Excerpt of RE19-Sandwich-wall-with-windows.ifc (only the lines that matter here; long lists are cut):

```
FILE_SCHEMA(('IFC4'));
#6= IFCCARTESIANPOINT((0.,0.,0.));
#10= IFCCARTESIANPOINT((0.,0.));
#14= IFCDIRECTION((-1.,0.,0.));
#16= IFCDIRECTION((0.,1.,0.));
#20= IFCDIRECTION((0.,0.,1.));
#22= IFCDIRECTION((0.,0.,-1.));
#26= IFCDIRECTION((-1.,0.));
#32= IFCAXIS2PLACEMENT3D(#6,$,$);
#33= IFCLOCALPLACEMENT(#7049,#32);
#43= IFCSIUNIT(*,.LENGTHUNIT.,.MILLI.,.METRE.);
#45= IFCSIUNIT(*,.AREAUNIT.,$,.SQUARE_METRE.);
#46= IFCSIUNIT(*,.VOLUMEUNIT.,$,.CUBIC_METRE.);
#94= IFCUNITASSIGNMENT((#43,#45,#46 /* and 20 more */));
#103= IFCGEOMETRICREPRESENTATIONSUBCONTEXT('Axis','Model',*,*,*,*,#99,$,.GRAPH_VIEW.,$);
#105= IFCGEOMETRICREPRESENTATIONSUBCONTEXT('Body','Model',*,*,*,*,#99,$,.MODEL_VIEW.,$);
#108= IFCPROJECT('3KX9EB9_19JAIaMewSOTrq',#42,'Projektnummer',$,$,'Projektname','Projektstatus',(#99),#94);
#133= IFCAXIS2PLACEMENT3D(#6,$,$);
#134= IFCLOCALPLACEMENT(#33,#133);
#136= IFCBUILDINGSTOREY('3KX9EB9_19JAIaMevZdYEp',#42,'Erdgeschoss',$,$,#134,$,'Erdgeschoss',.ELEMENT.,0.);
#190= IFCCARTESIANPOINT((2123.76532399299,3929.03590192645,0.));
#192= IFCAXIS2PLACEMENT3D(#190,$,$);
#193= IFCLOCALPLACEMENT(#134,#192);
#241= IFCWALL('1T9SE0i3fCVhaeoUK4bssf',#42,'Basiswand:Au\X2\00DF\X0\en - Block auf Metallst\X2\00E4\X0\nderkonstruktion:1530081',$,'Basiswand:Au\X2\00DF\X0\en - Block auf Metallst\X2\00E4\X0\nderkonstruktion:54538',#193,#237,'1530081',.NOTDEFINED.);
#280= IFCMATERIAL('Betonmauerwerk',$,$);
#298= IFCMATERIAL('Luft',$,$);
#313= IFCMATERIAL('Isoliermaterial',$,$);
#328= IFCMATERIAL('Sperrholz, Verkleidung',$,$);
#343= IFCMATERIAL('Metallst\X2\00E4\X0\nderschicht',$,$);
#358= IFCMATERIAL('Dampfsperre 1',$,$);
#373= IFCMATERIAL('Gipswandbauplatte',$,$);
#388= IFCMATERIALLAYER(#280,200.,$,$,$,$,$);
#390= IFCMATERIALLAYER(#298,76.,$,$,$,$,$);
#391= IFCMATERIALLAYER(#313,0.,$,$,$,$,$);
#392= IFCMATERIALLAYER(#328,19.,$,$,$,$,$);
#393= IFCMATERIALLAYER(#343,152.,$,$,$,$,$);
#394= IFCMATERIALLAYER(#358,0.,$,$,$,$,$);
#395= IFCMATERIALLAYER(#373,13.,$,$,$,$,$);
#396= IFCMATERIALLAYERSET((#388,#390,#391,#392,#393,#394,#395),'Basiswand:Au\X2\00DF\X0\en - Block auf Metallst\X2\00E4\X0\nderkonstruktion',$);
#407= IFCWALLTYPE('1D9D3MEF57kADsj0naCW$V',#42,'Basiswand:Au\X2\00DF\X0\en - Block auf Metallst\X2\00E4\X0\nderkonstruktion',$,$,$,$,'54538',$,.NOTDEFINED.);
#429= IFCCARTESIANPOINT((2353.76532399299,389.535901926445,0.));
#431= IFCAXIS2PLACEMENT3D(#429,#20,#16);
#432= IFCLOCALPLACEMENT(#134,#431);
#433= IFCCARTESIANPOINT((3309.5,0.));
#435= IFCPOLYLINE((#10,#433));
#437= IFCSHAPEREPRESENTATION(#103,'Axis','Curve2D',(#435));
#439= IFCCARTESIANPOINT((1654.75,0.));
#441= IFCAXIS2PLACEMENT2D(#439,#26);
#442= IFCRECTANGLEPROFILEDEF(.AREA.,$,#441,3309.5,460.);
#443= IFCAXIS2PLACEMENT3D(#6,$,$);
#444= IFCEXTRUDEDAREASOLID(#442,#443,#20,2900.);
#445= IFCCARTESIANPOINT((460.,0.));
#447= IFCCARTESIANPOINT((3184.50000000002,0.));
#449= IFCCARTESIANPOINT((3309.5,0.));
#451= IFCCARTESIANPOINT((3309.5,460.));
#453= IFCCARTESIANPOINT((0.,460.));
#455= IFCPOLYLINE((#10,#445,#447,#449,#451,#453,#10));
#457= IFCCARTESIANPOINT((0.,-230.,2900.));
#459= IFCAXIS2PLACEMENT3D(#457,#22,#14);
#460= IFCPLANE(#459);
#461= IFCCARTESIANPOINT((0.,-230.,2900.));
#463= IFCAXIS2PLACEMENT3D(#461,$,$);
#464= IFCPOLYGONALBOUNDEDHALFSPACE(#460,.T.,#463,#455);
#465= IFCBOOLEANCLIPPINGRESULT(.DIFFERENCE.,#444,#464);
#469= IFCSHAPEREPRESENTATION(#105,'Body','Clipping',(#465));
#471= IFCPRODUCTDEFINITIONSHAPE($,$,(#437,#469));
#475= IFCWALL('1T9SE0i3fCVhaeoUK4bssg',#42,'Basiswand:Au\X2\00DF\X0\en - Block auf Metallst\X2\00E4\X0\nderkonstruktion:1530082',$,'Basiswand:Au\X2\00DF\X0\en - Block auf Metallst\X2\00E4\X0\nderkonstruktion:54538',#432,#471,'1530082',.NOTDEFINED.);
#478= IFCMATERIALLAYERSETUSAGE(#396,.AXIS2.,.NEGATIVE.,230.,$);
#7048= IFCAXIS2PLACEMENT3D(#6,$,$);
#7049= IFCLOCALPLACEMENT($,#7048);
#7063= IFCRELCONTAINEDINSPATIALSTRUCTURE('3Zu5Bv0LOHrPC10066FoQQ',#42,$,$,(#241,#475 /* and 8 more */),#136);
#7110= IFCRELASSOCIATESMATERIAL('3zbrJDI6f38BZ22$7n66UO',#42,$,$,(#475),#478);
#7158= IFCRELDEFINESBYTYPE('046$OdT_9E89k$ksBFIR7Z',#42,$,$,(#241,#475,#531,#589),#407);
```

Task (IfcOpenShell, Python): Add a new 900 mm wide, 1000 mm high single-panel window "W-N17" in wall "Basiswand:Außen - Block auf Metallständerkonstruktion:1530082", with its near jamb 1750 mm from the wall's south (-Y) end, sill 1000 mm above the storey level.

```python
import numpy as np
import ifcopenshell
import ifcopenshell.api.feature
import ifcopenshell.api.geometry
import ifcopenshell.api.root
import ifcopenshell.api.spatial
import ifcopenshell.geom
import ifcopenshell.util.element
import ifcopenshell.util.placement
import ifcopenshell.util.representation
import ifcopenshell.util.shape
import ifcopenshell.util.unit

model = ifcopenshell.open("RE19-Sandwich-wall-with-windows.ifc")
unit_scale = ifcopenshell.util.unit.calculate_unit_scale(model)
settings = ifcopenshell.geom.settings()


def volume(element):
    """Net volume in cubic metres, openings subtracted."""
    shape = ifcopenshell.geom.create_shape(settings, element)
    return ifcopenshell.util.shape.get_volume(shape.geometry)


wall = model.by_guid("1T9SE0i3fCVhaeoUK4bssg")
storey = ifcopenshell.util.element.get_container(wall, ifc_class="IfcBuildingStorey")
context = ifcopenshell.util.representation.get_context(model, "Model", "Body", "MODEL_VIEW")
before = volume(wall)

width, height, from_end, sill = 0.9, 1, 1.75, 1  # metres

# The wall runs along its own X axis, and the end named is its -X end.
wall_shape = ifcopenshell.geom.create_shape(settings, wall)
x, y, z = ifcopenshell.util.shape.get_vertices(wall_shape.geometry).T
start = x.min() + from_end
face, thickness = float(y.min()), float(y.max() - y.min())
wall_matrix = ifcopenshell.util.placement.get_local_placement(wall.ObjectPlacement)
level = ifcopenshell.util.placement.get_local_placement(storey.ObjectPlacement)[2, 3]


def in_wall(x, y):
    """Placement at x, y metres in the wall's axes, at sill height."""
    matrix = wall_matrix.copy()
    matrix[:, 3] = wall_matrix @ np.array([x / unit_scale, y / unit_scale, 0.0, 1.0])
    matrix[2, 3] = level + sill / unit_scale
    return matrix


# Opening: a box that overshoots both wall faces by 50 mm.
opening = ifcopenshell.api.root.create_entity(model, ifc_class="IfcOpeningElement", predefined_type="OPENING")
box = ifcopenshell.api.geometry.add_wall_representation(
    model, context=context, length=width, height=height, thickness=thickness + 0.1
)
ifcopenshell.api.geometry.assign_representation(model, product=opening, representation=box)
ifcopenshell.api.geometry.edit_object_placement(model, product=opening, matrix=in_wall(start, face - 0.05), is_si=False)
ifcopenshell.api.feature.add_feature(model, feature=opening, element=wall)

window = ifcopenshell.api.root.create_entity(model, ifc_class="IfcWindow", name="W-N17", predefined_type="WINDOW")
window.OverallWidth, window.OverallHeight = width / unit_scale, height / unit_scale
window.PartitioningType = "SINGLE_PANEL"
body = ifcopenshell.api.geometry.add_window_representation(
    model,
    context=context,
    overall_width=window.OverallWidth,
    overall_height=window.OverallHeight,
    partition_type="SINGLE_PANEL",
)
ifcopenshell.api.geometry.assign_representation(model, product=window, representation=body)
ifcopenshell.api.spatial.assign_container(model, products=[window], relating_structure=storey)
ifcopenshell.api.feature.add_filling(model, opening=opening, element=window)

# Centre the window in the wall's thickness.
ifcopenshell.api.geometry.edit_object_placement(model, product=window, matrix=in_wall(start, face), is_si=False)
window_shape = ifcopenshell.geom.create_shape(settings, window)
depth = ifcopenshell.util.shape.get_vertices(window_shape.geometry)[:, 1]
offset = face + thickness / 2 - (depth.min() + depth.max()) / 2
ifcopenshell.api.geometry.edit_object_placement(model, product=window, matrix=in_wall(start, offset), is_si=False)

after = volume(wall)

print(f"wall volume {before:.3f} -> {after:.3f} m3")

model.write("RE19-Sandwich-wall-with-windows_updated.ifc")
```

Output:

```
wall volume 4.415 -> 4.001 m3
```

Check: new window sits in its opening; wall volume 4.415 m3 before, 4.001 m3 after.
